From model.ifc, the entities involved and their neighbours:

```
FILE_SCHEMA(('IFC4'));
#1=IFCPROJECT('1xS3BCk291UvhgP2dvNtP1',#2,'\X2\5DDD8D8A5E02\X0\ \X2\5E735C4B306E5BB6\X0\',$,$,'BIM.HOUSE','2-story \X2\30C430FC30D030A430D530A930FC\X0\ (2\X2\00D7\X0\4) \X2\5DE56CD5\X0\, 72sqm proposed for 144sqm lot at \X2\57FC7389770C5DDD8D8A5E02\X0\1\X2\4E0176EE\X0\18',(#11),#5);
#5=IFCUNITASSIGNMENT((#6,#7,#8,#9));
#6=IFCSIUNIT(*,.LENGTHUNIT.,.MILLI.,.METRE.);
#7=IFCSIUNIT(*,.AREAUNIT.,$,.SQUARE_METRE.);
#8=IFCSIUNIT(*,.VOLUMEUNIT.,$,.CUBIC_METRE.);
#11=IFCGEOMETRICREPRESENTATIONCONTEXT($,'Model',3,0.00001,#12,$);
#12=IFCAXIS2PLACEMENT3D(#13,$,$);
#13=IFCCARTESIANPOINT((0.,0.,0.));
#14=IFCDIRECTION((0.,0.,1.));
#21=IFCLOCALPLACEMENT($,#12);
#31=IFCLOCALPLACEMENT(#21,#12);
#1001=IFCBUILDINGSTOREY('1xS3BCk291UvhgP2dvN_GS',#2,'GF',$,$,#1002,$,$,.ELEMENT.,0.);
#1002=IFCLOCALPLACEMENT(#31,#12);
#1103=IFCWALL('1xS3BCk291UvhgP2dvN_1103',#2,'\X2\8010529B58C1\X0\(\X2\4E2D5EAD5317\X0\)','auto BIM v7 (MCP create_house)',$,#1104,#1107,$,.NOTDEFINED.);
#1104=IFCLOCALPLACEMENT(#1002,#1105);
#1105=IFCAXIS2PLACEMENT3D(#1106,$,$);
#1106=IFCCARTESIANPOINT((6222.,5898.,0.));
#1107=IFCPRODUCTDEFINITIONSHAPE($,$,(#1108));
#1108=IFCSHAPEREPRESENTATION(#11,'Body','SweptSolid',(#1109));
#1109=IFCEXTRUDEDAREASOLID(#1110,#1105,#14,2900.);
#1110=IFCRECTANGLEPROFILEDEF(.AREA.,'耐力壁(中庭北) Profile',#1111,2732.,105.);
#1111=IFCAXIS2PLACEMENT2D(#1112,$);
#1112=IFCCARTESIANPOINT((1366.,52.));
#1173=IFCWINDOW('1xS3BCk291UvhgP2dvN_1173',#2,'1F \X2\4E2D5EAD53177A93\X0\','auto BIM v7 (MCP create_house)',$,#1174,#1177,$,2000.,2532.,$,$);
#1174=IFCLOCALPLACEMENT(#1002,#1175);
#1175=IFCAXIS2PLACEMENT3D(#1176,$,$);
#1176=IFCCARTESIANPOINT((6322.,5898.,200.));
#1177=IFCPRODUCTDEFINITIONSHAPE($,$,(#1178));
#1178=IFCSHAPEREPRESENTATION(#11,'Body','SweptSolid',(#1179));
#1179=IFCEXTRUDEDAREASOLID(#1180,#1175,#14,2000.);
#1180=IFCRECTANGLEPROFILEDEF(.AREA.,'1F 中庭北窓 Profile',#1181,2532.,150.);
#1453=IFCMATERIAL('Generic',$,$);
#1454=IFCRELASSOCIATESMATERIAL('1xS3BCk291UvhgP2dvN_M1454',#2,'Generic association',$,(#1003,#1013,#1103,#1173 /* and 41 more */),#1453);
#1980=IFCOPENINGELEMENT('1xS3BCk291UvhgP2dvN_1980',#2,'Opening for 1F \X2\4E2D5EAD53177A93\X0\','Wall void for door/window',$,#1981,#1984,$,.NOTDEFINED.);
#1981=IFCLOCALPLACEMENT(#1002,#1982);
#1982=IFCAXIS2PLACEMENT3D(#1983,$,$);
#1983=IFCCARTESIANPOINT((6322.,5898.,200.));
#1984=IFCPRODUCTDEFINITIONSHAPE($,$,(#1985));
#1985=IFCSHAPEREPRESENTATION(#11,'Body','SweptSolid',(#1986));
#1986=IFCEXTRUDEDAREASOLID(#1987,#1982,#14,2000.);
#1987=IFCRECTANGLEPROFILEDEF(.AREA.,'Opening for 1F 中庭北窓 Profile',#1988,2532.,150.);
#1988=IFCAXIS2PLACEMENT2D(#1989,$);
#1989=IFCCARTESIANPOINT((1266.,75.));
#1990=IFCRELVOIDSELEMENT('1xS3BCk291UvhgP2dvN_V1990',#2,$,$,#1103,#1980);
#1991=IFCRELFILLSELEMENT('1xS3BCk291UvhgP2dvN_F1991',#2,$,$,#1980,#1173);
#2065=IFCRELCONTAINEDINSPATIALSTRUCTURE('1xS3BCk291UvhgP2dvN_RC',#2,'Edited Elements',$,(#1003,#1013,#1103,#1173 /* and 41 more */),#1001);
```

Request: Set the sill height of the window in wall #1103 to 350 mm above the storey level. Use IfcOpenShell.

```python
import numpy as np
import ifcopenshell
import ifcopenshell.api.geometry
import ifcopenshell.geom
import ifcopenshell.util.element
import ifcopenshell.util.placement
import ifcopenshell.util.shape
import ifcopenshell.util.unit

model = ifcopenshell.open("model.ifc")
unit_scale = ifcopenshell.util.unit.calculate_unit_scale(model)

window = model.by_guid("1xS3BCk291UvhgP2dvN_1173")
opening = window.FillsVoids[0].RelatingOpeningElement
storey = ifcopenshell.util.element.get_container(window, ifc_class="IfcBuildingStorey")
level = ifcopenshell.util.placement.get_local_placement(storey.ObjectPlacement)[2, 3]

# The opening's origin need not be at the sill, so measure its lowest point.
shape = ifcopenshell.geom.create_shape(ifcopenshell.geom.settings(), opening)
bottom = ifcopenshell.util.shape.get_shape_bottom_elevation(shape, shape.geometry) / unit_scale
dz = level + 0.35 / unit_scale - bottom

shift = np.array([0.0, 0.0, dz])
# The window is not placed relative to its opening, so move both.
for product in (opening, window):
    matrix = ifcopenshell.util.placement.get_local_placement(product.ObjectPlacement)
    matrix[:3, 3] += shift
    ifcopenshell.api.geometry.edit_object_placement(model, product=product, matrix=matrix, is_si=False)

print(f"moved by {dz * unit_scale:+.3f} m")

model.write("model_edited.ifc")
```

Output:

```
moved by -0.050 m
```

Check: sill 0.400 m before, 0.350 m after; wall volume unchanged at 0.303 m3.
